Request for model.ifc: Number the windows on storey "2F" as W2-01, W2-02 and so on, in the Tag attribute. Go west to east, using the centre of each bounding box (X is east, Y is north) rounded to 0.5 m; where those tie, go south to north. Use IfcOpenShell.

First a look at what the model holds.

```python
import ifcopenshell
import ifcopenshell.util.element
import ifcopenshell.util.placement

model = ifcopenshell.open("model.ifc")
print(model.schema)
storey = next(s for s in model.by_type("IfcBuildingStorey") if s.Name == "2F")
windows = [e for e in ifcopenshell.util.element.get_decomposition(storey) if e.is_a("IfcWindow")]
for e in sorted(windows, key=lambda e: e.id()):
    origin = ifcopenshell.util.placement.get_local_placement(e.ObjectPlacement)[:3, 3]
    print(e.id(), e.Tag, e.Name, origin.round(2) + 0.0, sep=" | ")
```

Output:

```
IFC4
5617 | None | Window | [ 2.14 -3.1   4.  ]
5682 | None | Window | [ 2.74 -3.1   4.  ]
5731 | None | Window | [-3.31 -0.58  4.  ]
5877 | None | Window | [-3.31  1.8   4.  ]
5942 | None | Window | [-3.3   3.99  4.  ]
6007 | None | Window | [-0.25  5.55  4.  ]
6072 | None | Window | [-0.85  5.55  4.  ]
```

```python
import ifcopenshell
import ifcopenshell.geom
import ifcopenshell.util.element
import ifcopenshell.util.shape

model = ifcopenshell.open("model.ifc")
settings = ifcopenshell.geom.settings()
settings.set("use-world-coords", True)


def centre(element):
    shape = ifcopenshell.geom.create_shape(settings, element)
    return ifcopenshell.util.shape.get_bbox_centroid(shape.geometry)


storey = next(s for s in model.by_type("IfcBuildingStorey") if s.Name == "2F")
windows = [e for e in ifcopenshell.util.element.get_decomposition(storey) if e.is_a("IfcWindow")]

# Insertion points can sit at a corner or the storey origin, so sort by the geometry (in metres).
centres = {e: centre(e) for e in windows}
windows.sort(key=lambda e: (round(centres[e][0] / 0.5), centres[e][1]))

for i, e in enumerate(windows, start=1):
    number = f"W2-{i:02d}"
    e.Tag = number
    print(e.id(), number)

model.write("model_edited.ifc")
```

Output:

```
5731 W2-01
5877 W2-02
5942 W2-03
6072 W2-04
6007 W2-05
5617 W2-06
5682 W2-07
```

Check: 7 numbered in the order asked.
